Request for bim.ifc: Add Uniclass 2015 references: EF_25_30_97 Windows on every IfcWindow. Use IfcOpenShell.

First a look at what the model holds.

```python
import ifcopenshell

model = ifcopenshell.open("bim.ifc")
print(model.schema)
print("classifications:", [c.Name for c in model.by_type("IfcClassification")])
for ifc_class in ("IfcDoor", "IfcRoof", "IfcStair", "IfcWall", "IfcWindow"):
    print(ifc_class, len(model.by_type(ifc_class)))
```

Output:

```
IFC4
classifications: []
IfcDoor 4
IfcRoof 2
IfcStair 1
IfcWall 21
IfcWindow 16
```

```python
import ifcopenshell
import ifcopenshell.api.classification

model = ifcopenshell.open("bim.ifc")

system = ifcopenshell.api.classification.add_classification(model, classification="Uniclass 2015")

codes = {
    "IfcWindow": ("EF_25_30_97", "Windows"),
}
for ifc_class, (code, name) in codes.items():
    products = model.by_type(ifc_class)
    ifcopenshell.api.classification.add_reference(
        model, products=products, classification=system, identification=code, name=name
    )
    print(code, len(products))

model.write("bim_updated.ifc")
```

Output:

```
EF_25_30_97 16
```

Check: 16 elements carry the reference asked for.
